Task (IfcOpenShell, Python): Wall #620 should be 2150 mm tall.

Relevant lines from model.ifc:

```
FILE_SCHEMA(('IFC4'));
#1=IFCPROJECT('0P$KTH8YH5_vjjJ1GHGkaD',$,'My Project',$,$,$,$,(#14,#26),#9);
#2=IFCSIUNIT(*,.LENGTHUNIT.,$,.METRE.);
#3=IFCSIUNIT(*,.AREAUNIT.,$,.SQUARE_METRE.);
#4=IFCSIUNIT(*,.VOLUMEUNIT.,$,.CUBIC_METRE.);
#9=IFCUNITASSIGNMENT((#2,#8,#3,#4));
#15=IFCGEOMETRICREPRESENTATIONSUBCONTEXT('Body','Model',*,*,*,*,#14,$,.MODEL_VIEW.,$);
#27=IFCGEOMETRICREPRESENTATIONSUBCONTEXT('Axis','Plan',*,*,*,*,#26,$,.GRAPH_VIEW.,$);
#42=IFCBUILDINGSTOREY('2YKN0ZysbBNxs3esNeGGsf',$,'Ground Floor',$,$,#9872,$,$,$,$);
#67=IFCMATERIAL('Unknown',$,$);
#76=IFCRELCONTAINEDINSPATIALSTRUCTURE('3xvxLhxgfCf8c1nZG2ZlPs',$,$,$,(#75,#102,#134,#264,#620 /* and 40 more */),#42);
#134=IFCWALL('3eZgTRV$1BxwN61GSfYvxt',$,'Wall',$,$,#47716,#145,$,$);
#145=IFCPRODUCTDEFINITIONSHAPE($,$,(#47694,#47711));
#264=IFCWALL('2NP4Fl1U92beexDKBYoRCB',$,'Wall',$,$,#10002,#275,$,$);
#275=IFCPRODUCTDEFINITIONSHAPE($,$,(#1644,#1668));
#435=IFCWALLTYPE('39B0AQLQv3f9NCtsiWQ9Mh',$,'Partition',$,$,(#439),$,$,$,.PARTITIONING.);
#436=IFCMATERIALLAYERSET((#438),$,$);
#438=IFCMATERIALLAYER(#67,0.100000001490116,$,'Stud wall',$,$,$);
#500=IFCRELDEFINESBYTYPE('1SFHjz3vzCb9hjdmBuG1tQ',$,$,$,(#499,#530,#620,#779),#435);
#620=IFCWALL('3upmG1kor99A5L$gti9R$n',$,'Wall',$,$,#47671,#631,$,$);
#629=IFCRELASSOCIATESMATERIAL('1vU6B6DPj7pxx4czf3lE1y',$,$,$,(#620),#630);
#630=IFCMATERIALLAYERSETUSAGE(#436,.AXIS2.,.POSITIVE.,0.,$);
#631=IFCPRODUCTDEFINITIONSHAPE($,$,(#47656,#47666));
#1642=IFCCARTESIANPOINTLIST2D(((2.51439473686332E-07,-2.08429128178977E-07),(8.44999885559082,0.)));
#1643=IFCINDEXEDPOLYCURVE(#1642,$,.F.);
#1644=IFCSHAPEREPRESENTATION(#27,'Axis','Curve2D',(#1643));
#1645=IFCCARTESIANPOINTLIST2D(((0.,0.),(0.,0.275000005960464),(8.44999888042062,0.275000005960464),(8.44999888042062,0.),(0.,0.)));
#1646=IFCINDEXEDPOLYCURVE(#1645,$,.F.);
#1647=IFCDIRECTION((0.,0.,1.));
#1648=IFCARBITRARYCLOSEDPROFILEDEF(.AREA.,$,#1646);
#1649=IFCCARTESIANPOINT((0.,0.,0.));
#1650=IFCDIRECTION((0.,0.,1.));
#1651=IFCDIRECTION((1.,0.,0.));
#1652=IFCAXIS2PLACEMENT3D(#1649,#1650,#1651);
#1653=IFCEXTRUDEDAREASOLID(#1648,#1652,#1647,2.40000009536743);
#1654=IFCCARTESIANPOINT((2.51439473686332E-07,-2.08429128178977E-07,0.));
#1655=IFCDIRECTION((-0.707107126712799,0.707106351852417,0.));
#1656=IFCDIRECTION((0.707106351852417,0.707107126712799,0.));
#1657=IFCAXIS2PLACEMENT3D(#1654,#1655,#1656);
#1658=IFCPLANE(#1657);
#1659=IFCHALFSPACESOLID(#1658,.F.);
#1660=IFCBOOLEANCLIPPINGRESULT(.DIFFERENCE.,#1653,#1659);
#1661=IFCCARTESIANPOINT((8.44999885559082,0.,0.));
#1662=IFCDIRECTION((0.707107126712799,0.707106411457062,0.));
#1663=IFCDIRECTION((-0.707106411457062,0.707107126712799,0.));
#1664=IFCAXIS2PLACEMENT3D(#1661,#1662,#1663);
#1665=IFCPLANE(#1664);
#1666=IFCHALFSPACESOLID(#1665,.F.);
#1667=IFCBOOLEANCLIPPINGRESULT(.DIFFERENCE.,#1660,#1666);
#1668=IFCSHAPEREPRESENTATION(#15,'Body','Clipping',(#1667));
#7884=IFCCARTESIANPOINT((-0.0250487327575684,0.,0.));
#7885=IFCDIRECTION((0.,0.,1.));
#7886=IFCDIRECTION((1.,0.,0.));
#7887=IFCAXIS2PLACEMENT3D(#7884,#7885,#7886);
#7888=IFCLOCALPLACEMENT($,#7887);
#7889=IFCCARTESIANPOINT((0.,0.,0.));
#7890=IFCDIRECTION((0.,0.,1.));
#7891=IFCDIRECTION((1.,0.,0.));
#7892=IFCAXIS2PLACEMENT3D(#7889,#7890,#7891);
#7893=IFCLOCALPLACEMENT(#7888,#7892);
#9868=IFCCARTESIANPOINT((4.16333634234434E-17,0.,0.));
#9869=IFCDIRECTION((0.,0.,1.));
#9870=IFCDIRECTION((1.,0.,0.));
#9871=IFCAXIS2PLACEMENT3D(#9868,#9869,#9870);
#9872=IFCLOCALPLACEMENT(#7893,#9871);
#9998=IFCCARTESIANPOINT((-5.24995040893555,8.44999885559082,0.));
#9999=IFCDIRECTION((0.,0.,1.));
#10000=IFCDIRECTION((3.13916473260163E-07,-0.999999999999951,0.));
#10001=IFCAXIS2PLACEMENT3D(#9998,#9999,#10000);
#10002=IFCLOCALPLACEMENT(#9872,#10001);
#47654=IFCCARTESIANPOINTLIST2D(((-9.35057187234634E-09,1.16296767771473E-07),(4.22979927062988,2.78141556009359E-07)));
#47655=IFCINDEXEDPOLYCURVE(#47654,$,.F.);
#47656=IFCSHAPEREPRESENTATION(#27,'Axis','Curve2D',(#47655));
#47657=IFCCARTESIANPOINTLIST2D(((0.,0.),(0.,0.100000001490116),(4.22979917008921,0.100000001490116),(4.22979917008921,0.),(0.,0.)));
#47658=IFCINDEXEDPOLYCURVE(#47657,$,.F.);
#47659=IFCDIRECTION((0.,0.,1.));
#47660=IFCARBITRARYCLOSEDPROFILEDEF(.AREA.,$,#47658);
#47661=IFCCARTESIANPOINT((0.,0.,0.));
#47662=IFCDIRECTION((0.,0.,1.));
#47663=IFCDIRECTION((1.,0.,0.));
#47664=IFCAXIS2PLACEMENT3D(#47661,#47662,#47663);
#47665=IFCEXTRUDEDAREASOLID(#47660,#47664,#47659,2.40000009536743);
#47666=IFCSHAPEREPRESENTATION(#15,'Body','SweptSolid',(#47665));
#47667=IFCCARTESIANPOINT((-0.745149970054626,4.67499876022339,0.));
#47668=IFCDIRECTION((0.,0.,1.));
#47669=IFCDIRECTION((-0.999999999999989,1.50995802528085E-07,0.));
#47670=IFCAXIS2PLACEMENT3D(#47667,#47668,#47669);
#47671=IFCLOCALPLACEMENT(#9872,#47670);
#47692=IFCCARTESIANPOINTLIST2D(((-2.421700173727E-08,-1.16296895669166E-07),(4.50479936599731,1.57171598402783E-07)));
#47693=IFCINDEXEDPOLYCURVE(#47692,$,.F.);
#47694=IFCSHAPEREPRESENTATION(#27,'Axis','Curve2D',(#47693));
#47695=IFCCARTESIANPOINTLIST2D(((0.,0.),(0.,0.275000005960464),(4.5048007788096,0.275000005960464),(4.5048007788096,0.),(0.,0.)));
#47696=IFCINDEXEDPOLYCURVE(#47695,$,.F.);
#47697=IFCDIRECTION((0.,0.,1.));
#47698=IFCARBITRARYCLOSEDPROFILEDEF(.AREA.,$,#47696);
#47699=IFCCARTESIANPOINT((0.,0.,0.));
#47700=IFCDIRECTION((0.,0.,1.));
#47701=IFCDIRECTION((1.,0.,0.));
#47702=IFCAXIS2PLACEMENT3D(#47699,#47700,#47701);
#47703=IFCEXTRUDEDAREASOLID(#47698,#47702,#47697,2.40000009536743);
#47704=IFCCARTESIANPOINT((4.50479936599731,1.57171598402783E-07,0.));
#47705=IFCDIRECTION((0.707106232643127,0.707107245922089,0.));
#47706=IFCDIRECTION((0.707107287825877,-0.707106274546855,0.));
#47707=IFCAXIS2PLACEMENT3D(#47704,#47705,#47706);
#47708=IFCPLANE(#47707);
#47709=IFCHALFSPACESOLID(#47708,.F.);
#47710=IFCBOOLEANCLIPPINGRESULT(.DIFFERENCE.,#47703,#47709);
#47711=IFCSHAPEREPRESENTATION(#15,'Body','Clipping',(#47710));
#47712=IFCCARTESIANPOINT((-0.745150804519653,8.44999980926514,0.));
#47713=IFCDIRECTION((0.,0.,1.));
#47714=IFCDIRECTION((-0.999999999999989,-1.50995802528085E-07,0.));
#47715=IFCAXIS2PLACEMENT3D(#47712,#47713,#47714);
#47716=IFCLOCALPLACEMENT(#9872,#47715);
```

```python
import ifcopenshell
import ifcopenshell.geom
import ifcopenshell.util.representation
import ifcopenshell.util.shape

model = ifcopenshell.open("model.ifc")
settings = ifcopenshell.geom.settings()


def volume(element):
    """Net volume in cubic metres, openings subtracted."""
    shape = ifcopenshell.geom.create_shape(settings, element)
    return ifcopenshell.util.shape.get_volume(shape.geometry)


wall = model.by_guid("3upmG1kor99A5L$gti9R$n")
before = volume(wall)

body = ifcopenshell.util.representation.get_representation(wall, "Model", "Body")
solid = body.Items[0]
old_height = solid.Depth
solid.Depth = 2.15
after = volume(wall)

print(f"height {old_height:g} -> {solid.Depth:g}, volume {before:.3f} -> {after:.3f} m3")

model.write("model_v2.ifc")
```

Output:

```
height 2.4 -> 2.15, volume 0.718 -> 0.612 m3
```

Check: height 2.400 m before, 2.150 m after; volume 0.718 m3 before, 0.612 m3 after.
